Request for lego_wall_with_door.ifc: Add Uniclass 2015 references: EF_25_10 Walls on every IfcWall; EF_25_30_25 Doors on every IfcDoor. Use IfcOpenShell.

First a look at what the model holds.

```python
import ifcopenshell

model = ifcopenshell.open("lego_wall_with_door.ifc")
print(model.schema)
print("classifications:", [c.Name for c in model.by_type("IfcClassification")])
for ifc_class in ("IfcDoor", "IfcRoof", "IfcStair", "IfcWall", "IfcWindow"):
    print(ifc_class, len(model.by_type(ifc_class)))
```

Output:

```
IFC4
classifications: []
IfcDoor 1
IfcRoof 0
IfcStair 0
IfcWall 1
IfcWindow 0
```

```python
import ifcopenshell
import ifcopenshell.api.classification

model = ifcopenshell.open("lego_wall_with_door.ifc")

system = ifcopenshell.api.classification.add_classification(model, classification="Uniclass 2015")

codes = {
    "IfcWall": ("EF_25_10", "Walls"),
    "IfcDoor": ("EF_25_30_25", "Doors"),
}
for ifc_class, (code, name) in codes.items():
    products = model.by_type(ifc_class)
    ifcopenshell.api.classification.add_reference(
        model, products=products, classification=system, identification=code, name=name
    )
    print(code, len(products))

model.write("lego_wall_with_door_updated.ifc")
```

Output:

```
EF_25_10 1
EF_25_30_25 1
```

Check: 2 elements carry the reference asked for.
